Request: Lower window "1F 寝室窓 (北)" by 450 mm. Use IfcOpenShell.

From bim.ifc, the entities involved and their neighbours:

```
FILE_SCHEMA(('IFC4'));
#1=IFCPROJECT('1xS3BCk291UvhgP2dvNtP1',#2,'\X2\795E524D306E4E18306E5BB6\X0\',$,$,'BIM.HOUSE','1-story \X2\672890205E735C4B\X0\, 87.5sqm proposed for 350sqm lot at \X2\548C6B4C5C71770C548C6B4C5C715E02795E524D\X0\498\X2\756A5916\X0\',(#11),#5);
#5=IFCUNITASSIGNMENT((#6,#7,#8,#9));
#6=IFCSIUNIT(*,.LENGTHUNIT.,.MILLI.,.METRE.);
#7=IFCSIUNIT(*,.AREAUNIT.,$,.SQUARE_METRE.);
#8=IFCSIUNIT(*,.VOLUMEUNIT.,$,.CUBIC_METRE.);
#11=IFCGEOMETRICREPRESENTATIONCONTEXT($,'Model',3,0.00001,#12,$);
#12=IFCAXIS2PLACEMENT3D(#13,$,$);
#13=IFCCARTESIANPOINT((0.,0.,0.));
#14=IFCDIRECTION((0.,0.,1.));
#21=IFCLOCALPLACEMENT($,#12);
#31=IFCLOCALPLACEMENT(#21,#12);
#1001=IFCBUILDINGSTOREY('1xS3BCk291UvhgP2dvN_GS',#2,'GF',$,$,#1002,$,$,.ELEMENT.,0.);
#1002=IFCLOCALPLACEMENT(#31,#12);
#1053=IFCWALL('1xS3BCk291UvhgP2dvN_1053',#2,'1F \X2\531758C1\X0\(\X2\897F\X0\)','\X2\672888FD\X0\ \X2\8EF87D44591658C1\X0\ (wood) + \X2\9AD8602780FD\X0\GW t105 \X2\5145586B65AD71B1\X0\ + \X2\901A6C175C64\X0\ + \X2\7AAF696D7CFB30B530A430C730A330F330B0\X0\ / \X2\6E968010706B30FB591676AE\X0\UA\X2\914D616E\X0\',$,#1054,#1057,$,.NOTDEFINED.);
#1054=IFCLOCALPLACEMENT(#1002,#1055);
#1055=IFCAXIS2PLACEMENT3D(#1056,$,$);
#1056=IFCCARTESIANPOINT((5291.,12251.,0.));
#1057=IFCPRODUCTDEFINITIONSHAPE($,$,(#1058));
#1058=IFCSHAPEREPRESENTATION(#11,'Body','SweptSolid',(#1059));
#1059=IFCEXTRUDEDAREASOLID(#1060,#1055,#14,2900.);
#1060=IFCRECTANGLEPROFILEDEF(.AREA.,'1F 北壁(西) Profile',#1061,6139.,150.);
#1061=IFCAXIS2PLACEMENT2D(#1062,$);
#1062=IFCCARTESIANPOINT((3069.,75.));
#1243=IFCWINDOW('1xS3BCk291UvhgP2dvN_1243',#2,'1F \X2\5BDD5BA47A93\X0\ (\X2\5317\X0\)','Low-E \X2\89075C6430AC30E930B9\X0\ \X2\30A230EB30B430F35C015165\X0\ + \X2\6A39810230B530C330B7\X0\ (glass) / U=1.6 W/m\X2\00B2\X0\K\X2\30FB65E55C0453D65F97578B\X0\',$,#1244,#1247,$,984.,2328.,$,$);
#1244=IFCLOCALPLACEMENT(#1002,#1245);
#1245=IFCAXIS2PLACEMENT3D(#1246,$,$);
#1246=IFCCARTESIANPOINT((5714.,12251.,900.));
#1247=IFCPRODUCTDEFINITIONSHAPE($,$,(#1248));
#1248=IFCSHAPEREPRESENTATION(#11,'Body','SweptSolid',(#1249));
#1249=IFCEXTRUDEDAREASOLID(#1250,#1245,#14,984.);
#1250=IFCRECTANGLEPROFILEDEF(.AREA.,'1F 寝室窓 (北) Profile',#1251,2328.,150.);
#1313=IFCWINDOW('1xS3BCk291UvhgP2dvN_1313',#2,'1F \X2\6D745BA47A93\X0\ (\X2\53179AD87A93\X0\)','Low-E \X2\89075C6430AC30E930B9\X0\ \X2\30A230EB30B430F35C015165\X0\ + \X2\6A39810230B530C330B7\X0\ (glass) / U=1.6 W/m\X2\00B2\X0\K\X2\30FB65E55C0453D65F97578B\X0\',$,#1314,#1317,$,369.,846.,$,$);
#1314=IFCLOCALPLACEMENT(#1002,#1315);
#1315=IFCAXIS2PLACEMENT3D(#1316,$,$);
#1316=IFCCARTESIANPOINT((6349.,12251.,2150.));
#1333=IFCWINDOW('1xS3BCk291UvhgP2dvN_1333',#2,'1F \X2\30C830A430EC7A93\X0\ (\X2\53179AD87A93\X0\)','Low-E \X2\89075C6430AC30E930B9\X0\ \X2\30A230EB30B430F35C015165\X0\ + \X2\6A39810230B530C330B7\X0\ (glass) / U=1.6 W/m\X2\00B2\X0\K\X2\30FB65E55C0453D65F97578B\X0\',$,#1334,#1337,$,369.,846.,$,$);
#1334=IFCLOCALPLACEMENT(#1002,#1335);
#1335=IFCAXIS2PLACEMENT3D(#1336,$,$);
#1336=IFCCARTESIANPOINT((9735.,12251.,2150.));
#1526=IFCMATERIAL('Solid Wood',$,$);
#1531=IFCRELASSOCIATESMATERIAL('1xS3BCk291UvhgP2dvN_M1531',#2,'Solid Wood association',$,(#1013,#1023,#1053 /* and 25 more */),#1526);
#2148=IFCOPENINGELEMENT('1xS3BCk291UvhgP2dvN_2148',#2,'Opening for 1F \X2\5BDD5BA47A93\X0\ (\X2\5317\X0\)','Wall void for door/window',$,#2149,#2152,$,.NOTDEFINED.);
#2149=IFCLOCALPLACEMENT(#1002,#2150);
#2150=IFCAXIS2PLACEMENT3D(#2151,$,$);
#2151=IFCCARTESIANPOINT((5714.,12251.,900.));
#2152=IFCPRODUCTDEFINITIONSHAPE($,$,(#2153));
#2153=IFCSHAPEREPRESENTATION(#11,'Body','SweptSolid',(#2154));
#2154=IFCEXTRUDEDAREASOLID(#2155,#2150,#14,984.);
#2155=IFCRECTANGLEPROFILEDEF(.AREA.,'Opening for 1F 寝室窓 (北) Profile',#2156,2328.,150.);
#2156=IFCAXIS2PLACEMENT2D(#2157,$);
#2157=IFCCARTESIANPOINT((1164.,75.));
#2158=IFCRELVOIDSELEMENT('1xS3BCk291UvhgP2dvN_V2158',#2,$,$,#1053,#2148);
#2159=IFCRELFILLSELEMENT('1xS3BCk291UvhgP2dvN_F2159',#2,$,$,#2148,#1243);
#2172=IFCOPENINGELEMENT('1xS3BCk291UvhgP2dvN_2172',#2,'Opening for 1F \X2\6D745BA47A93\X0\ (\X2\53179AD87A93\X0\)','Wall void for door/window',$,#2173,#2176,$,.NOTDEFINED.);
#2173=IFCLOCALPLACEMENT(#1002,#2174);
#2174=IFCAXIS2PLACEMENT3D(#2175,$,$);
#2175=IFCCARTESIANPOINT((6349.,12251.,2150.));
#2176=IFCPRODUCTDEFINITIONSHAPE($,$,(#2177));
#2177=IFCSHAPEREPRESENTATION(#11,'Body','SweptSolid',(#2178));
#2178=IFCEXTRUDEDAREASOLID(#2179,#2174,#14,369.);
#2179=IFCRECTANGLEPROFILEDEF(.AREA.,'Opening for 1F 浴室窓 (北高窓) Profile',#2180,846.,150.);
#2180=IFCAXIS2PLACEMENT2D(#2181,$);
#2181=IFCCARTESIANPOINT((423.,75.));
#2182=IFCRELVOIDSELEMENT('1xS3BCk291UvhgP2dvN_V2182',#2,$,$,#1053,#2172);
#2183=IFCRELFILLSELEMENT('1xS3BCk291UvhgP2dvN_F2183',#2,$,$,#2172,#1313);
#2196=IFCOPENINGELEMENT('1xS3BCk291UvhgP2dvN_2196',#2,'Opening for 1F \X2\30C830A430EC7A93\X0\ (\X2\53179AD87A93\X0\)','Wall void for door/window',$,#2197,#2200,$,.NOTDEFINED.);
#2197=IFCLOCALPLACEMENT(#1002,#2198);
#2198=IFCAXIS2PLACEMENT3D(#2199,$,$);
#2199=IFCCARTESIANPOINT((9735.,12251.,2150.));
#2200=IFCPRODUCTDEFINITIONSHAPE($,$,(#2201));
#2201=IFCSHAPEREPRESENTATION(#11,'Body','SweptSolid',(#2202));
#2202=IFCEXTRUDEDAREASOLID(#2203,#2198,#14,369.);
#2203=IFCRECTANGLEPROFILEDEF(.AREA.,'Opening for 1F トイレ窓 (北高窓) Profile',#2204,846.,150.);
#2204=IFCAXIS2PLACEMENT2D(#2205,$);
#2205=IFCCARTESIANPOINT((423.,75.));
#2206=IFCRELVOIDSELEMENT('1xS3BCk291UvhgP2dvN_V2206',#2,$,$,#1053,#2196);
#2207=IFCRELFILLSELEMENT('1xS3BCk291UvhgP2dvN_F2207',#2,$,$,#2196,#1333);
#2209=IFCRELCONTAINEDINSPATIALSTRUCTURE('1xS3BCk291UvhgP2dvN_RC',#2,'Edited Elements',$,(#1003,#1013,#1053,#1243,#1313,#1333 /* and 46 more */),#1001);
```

```python
import numpy as np
import ifcopenshell
import ifcopenshell.api.geometry
import ifcopenshell.util.placement
import ifcopenshell.util.unit

model = ifcopenshell.open("bim.ifc")
unit_scale = ifcopenshell.util.unit.calculate_unit_scale(model)

window = model.by_guid("1xS3BCk291UvhgP2dvN_1243")
opening = window.FillsVoids[0].RelatingOpeningElement
dz = -0.45 / unit_scale

shift = np.array([0.0, 0.0, dz])
# The window is not placed relative to its opening, so move both.
for product in (opening, window):
    matrix = ifcopenshell.util.placement.get_local_placement(product.ObjectPlacement)
    matrix[:3, 3] += shift
    ifcopenshell.api.geometry.edit_object_placement(model, product=product, matrix=matrix, is_si=False)

print(f"moved by {dz * unit_scale:+.3f} m")

model.write("bim_updated.ifc")
```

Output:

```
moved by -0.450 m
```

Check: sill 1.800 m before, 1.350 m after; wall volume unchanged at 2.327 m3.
